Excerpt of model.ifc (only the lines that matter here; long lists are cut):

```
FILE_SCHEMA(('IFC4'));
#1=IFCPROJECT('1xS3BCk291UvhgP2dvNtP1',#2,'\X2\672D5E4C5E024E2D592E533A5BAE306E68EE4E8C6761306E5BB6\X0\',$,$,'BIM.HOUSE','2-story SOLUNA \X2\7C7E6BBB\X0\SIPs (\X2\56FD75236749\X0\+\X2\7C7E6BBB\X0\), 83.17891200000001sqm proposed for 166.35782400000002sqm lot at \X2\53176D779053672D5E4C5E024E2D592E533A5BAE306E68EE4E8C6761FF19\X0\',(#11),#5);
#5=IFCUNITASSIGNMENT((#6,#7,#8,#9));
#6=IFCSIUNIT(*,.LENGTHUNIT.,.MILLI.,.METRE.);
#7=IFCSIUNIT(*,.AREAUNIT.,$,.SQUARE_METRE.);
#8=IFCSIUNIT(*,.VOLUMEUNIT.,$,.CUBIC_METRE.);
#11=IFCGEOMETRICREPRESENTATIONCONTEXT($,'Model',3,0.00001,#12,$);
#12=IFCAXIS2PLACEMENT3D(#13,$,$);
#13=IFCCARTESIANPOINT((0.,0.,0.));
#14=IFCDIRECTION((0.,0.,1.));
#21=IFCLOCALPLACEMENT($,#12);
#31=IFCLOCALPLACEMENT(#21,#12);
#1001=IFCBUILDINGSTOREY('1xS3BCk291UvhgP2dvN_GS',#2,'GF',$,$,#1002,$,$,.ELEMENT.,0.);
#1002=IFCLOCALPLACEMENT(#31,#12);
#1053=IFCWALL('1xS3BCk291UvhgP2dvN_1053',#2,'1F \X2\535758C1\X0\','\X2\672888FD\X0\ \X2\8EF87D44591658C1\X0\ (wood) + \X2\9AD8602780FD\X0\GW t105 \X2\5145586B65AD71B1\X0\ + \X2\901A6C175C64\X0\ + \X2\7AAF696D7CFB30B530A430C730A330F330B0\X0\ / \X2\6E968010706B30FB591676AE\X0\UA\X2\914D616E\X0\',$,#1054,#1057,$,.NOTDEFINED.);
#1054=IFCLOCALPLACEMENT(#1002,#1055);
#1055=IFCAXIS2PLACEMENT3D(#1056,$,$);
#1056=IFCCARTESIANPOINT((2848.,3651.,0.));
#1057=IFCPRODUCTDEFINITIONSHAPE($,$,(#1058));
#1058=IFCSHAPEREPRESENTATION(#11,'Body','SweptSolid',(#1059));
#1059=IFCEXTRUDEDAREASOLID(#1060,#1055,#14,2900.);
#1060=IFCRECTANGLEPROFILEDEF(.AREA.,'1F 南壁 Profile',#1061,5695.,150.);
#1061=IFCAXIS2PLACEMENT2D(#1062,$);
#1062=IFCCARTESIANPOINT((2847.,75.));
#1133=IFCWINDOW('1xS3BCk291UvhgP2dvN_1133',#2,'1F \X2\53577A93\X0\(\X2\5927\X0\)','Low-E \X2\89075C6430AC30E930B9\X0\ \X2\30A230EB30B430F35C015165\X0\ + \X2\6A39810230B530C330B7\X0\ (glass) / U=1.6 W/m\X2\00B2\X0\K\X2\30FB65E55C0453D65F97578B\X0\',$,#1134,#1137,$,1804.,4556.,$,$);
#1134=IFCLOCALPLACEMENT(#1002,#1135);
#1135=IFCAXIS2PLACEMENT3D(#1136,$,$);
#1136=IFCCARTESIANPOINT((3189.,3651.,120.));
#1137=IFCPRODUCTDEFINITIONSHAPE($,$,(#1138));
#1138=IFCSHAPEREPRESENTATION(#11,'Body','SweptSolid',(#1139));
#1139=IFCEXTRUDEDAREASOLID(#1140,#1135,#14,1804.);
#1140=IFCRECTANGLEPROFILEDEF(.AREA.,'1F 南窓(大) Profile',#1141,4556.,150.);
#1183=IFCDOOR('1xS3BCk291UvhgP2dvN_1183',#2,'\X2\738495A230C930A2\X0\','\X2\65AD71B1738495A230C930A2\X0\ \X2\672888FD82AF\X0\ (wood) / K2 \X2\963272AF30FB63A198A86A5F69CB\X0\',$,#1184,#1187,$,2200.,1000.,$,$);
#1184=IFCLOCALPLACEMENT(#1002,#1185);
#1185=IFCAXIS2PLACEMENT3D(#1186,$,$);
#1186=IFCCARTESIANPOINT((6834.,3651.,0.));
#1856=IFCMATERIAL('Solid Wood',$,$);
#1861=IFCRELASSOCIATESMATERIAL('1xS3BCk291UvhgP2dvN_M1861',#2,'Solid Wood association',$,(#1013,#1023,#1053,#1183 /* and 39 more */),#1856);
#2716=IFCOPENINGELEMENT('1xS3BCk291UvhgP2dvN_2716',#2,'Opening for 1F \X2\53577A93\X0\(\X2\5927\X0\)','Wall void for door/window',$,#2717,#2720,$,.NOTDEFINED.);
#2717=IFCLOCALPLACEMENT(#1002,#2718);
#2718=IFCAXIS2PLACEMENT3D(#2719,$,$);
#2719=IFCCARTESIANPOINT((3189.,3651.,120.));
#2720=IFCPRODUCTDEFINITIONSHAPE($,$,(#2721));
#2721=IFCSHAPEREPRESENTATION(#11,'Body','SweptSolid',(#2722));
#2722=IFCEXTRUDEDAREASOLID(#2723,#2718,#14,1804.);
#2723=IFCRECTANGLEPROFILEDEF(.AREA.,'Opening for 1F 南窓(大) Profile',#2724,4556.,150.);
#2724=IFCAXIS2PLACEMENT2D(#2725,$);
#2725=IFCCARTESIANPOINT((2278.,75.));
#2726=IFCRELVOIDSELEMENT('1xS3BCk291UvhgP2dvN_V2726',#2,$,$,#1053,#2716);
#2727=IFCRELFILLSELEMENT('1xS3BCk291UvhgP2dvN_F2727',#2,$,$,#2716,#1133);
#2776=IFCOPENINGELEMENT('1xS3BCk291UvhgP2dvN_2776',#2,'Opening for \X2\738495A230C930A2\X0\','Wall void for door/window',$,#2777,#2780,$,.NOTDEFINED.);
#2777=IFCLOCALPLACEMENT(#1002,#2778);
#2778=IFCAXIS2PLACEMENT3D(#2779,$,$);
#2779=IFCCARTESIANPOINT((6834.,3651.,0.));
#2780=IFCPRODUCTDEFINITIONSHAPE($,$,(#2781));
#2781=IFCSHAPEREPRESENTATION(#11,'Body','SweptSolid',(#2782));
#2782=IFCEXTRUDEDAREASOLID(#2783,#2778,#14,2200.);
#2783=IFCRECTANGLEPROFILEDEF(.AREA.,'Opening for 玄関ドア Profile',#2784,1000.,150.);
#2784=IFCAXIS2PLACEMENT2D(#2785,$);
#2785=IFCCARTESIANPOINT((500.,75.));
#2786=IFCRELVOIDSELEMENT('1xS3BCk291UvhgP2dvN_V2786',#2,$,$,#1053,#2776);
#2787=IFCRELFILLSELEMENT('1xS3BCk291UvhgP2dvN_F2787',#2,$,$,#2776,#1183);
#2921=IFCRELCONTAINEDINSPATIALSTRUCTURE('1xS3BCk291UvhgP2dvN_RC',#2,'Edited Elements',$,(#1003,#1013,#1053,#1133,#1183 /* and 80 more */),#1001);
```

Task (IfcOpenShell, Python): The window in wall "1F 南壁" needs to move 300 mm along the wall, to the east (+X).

```python
import ifcopenshell
import ifcopenshell.api.geometry
import ifcopenshell.util.placement

model = ifcopenshell.open("model.ifc")

window = model.by_guid("1xS3BCk291UvhgP2dvN_1133")
opening = window.FillsVoids[0].RelatingOpeningElement
wall = opening.VoidsElements[0].RelatingBuildingElement

wall_matrix = ifcopenshell.util.placement.get_local_placement(wall.ObjectPlacement)
shift = wall_matrix[:3, 0] * 300.0
before = ifcopenshell.util.placement.get_local_placement(window.ObjectPlacement)[:3, 3].copy()

# The window is not placed relative to its opening, so move both.
for product in (opening, window):
    matrix = ifcopenshell.util.placement.get_local_placement(product.ObjectPlacement)
    matrix[:3, 3] += shift
    ifcopenshell.api.geometry.edit_object_placement(model, product=product, matrix=matrix, is_si=False)

after = ifcopenshell.util.placement.get_local_placement(window.ObjectPlacement)[:3, 3]
print("window moved by", (after - before).round(3) + 0.0)

model.write("model_v2.ifc")
```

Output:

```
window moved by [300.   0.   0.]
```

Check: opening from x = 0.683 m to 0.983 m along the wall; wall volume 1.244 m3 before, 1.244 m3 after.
